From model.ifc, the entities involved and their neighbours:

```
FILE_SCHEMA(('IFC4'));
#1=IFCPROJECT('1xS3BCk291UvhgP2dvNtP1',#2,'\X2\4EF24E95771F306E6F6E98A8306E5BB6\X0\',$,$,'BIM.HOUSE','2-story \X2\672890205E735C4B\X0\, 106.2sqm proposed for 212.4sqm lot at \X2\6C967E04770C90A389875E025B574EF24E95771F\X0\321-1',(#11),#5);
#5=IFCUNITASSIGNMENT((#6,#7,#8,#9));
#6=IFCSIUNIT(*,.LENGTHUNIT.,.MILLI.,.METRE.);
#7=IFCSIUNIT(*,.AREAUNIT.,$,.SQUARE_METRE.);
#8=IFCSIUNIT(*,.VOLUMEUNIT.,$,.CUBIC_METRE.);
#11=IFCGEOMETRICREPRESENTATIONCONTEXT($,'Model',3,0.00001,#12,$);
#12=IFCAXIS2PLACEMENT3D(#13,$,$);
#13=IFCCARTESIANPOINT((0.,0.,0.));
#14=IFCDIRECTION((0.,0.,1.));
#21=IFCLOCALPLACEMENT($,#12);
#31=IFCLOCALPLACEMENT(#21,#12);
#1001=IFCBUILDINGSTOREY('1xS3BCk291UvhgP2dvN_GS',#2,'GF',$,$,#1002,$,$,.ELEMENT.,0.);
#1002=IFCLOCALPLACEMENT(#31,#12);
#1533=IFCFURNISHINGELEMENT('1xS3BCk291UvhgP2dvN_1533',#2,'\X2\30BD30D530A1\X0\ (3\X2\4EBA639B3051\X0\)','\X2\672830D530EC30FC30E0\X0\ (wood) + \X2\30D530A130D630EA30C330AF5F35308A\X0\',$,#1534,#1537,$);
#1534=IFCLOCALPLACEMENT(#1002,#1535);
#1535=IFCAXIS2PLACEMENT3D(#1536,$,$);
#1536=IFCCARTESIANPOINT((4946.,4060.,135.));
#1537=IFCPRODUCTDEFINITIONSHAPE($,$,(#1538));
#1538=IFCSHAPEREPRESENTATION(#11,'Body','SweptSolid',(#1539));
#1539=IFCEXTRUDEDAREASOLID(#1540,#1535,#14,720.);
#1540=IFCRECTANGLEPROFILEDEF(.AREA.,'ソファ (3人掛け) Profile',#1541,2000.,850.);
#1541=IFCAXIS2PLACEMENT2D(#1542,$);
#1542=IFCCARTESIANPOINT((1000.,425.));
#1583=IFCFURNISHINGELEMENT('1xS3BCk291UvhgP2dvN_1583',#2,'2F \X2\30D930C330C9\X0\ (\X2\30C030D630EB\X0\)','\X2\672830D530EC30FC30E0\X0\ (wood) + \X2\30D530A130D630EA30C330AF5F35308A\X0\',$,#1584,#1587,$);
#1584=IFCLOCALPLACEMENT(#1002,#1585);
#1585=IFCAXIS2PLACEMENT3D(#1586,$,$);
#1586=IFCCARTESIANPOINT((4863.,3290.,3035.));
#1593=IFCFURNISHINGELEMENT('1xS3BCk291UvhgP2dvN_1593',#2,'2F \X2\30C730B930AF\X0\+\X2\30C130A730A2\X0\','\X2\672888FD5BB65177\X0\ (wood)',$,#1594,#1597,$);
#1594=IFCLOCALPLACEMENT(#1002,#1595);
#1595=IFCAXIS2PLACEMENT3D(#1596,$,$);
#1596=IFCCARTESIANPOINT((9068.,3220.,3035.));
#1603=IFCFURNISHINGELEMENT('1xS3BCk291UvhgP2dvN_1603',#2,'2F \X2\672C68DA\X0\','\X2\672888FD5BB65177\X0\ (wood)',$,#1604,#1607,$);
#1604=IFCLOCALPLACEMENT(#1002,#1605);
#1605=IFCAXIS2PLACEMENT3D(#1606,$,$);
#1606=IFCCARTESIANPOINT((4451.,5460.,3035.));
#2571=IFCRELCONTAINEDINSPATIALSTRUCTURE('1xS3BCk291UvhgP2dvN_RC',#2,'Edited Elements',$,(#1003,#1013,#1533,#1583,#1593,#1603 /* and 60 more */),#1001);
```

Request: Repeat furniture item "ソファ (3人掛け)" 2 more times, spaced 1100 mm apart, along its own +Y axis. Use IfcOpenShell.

```python
import ifcopenshell
import ifcopenshell.api.geometry
import ifcopenshell.api.root
import ifcopenshell.util.element
import ifcopenshell.util.placement
import ifcopenshell.util.unit

model = ifcopenshell.open("model.ifc")
unit_scale = ifcopenshell.util.unit.calculate_unit_scale(model)


def reuse_history(source, copy):
    """copy_class also copies each property set's owner history, people and application; keep the originals."""
    for rel in copy.IsDefinedBy:
        if rel.is_a("IfcRelDefinesByProperties") and (history := rel.RelatingPropertyDefinition.OwnerHistory):
            rel.RelatingPropertyDefinition.OwnerHistory = source.OwnerHistory
            ifcopenshell.util.element.remove_deep2(model, history)


source = model.by_guid("1xS3BCk291UvhgP2dvN_1533")
base = ifcopenshell.util.placement.get_local_placement(source.ObjectPlacement)
step = base[:3, 1] * 1.1 / unit_scale

for i in range(1, 3):
    copy = ifcopenshell.api.root.copy_class(model, product=source)
    copy.Representation = ifcopenshell.util.element.copy_deep(
        model, source.Representation, exclude=["IfcGeometricRepresentationContext", "IfcRepresentationMap"]
    )
    reuse_history(source, copy)
    matrix = base.copy()
    matrix[:3, 3] += i * step
    print("added at", matrix[:3, 3].round(3) + 0.0)
    ifcopenshell.api.geometry.edit_object_placement(model, product=copy, matrix=matrix, is_si=False)

model.write("model_rev.ifc")
```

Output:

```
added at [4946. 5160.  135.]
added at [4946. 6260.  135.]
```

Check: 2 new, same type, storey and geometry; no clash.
